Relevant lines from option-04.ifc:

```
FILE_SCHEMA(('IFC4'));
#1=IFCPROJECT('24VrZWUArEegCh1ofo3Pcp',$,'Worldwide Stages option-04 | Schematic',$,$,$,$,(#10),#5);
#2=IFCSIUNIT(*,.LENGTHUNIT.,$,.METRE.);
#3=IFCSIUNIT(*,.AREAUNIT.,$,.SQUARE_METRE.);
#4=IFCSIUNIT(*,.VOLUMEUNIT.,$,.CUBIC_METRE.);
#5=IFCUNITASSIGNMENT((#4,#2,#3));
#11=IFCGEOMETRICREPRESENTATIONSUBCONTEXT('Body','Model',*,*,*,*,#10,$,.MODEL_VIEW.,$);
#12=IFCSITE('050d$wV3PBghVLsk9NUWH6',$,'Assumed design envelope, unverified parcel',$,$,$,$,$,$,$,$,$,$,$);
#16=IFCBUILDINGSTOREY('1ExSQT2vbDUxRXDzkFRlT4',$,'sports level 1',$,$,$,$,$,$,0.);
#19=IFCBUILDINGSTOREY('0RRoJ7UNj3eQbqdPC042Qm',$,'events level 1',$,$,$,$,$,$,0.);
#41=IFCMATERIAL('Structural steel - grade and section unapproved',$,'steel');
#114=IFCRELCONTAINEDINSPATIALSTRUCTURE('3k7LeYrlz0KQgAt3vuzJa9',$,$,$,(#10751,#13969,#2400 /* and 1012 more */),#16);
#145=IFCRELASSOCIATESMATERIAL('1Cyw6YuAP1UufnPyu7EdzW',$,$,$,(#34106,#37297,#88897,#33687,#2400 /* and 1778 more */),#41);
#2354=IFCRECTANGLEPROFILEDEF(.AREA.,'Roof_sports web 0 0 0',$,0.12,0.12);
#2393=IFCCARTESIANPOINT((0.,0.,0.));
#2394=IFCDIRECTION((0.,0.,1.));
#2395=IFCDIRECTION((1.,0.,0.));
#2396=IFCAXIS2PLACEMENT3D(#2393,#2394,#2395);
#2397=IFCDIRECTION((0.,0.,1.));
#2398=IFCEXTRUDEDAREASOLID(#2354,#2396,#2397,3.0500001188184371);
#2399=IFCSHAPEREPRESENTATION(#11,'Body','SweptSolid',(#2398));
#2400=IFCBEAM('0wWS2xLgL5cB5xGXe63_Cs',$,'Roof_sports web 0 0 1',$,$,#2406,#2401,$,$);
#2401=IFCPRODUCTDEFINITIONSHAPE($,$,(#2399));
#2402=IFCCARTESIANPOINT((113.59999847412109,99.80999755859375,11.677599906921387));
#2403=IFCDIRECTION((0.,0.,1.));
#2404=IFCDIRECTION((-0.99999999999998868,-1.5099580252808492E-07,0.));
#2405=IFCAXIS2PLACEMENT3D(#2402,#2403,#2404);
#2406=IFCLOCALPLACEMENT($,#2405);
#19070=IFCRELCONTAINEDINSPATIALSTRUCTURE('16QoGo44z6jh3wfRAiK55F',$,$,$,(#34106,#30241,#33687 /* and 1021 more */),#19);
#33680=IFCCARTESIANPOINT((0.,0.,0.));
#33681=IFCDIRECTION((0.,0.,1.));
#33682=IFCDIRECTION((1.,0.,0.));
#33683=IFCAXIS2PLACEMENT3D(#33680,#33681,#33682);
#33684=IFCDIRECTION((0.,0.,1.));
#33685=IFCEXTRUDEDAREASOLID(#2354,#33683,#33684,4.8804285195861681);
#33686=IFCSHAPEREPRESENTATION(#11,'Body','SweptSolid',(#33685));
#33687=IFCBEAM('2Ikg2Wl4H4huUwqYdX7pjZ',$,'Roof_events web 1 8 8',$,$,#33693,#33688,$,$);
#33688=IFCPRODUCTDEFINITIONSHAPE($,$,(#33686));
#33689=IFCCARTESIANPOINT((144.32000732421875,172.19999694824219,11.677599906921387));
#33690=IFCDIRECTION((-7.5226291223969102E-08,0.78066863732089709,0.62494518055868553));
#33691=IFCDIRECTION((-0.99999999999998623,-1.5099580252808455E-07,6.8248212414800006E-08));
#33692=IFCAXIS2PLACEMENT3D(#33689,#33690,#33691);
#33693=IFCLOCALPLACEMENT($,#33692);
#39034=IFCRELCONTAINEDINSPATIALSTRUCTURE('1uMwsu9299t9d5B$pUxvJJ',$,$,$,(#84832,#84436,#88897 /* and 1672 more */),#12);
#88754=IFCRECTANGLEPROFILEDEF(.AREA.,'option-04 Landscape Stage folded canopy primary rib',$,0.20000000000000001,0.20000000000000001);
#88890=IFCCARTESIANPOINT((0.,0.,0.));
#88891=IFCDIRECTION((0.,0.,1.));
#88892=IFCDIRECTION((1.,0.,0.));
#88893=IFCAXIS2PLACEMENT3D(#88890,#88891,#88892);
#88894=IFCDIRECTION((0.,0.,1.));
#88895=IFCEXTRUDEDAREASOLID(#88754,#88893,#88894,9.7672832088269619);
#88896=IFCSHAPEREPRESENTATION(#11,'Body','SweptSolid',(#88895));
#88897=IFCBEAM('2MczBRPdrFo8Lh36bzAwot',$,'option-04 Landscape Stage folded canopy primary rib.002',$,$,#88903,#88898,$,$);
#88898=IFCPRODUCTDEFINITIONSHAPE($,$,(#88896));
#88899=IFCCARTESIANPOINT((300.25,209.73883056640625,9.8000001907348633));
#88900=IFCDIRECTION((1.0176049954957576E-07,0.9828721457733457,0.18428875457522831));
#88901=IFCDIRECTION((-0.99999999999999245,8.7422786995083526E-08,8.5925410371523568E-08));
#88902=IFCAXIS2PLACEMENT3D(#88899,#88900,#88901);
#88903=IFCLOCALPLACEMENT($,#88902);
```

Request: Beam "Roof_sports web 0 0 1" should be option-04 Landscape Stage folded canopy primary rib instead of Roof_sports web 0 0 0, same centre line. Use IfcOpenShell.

```python
import ifcopenshell
import ifcopenshell.util.element
import ifcopenshell.util.representation

model = ifcopenshell.open("option-04.ifc")

member = model.by_guid("0wWS2xLgL5cB5xGXe63_Cs")
source = next(p for p in model.by_type("IfcRectangleProfileDef") if p.ProfileName == "option-04 Landscape Stage folded canopy primary rib")

body = ifcopenshell.util.representation.get_representation(member, "Model", "Body")
solid = body.Items[0]
old_profile = solid.SweptArea

# Copy the section's sizes but keep this member's own profile position.
profile = ifcopenshell.util.element.copy(model, source)
profile.Position = old_profile.Position
solid.SweptArea = profile
if not model.get_total_inverses(old_profile):
    ifcopenshell.util.element.remove_deep2(model, old_profile)

print(solid.SweptArea)

model.write("option-04_v2.ifc")
```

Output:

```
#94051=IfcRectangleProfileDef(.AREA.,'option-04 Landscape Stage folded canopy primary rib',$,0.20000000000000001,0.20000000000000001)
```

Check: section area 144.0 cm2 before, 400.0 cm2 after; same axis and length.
